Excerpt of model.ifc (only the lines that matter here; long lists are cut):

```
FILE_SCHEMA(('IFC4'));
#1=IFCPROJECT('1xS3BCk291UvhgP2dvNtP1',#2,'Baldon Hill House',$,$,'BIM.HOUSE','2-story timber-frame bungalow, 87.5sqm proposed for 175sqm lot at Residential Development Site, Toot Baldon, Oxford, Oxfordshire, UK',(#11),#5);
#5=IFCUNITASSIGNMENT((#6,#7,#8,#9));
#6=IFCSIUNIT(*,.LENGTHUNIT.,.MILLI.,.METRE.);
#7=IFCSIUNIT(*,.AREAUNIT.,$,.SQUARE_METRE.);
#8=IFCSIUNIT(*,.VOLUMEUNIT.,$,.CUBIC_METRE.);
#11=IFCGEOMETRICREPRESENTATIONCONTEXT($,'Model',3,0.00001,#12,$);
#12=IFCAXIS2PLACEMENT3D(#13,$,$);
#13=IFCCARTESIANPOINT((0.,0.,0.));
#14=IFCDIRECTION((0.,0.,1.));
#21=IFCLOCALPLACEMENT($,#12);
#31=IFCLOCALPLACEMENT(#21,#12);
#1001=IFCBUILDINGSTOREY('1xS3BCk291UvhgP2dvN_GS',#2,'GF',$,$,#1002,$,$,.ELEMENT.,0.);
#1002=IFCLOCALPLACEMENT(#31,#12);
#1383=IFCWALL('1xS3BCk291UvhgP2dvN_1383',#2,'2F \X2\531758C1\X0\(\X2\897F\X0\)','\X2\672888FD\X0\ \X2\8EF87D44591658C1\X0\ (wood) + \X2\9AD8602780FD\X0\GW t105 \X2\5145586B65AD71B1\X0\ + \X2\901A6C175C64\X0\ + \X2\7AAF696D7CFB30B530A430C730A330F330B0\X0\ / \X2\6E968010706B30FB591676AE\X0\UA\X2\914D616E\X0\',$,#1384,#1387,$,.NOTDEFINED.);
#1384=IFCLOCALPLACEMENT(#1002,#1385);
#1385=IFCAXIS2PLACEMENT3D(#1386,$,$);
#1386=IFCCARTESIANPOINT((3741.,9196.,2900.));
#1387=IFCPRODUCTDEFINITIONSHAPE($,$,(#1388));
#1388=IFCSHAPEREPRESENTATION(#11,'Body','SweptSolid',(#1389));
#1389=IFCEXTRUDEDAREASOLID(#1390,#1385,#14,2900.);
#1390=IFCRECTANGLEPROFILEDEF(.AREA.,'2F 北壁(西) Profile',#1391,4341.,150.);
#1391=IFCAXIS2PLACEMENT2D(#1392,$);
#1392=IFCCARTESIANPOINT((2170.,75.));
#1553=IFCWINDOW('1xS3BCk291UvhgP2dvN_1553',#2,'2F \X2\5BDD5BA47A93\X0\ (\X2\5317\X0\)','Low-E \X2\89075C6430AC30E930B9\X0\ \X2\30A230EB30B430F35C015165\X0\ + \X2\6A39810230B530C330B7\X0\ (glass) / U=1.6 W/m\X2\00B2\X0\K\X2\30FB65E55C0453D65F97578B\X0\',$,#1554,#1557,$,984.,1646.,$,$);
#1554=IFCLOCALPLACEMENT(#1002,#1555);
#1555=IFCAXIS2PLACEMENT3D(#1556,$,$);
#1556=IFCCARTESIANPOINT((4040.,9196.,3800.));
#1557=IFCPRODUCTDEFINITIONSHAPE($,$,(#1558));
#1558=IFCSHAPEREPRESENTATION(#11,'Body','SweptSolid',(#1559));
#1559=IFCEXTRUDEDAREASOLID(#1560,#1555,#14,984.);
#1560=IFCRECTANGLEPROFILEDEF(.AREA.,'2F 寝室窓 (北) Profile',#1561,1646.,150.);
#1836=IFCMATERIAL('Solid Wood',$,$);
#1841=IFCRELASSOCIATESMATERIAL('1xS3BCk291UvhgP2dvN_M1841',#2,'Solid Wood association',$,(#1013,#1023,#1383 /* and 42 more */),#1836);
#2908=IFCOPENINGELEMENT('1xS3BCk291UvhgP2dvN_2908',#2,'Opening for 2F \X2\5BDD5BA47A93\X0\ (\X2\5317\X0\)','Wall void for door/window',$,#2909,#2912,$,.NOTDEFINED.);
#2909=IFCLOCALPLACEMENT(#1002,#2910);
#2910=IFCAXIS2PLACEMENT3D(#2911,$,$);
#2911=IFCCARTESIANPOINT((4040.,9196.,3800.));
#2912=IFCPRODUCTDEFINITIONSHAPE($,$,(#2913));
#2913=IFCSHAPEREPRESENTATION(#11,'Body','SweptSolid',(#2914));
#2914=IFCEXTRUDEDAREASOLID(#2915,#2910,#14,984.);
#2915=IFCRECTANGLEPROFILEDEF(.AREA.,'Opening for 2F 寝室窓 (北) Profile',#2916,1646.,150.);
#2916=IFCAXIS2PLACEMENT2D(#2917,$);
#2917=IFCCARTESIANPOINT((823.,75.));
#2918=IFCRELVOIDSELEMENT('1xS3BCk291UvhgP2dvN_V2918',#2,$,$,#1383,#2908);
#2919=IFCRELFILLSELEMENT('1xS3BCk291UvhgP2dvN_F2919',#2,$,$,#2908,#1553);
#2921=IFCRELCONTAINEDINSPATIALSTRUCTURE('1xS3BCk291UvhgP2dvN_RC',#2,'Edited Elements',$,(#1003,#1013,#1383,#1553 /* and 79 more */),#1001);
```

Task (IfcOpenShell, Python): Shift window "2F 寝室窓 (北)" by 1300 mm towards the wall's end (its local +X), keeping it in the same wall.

```python
import ifcopenshell
import ifcopenshell.api.geometry
import ifcopenshell.util.placement

model = ifcopenshell.open("model.ifc")

window = model.by_guid("1xS3BCk291UvhgP2dvN_1553")
opening = window.FillsVoids[0].RelatingOpeningElement
wall = opening.VoidsElements[0].RelatingBuildingElement

wall_matrix = ifcopenshell.util.placement.get_local_placement(wall.ObjectPlacement)
shift = wall_matrix[:3, 0] * 1300.0
before = ifcopenshell.util.placement.get_local_placement(window.ObjectPlacement)[:3, 3].copy()

# The window is not placed relative to its opening, so move both.
for product in (opening, window):
    matrix = ifcopenshell.util.placement.get_local_placement(product.ObjectPlacement)
    matrix[:3, 3] += shift
    ifcopenshell.api.geometry.edit_object_placement(model, product=product, matrix=matrix, is_si=False)

after = ifcopenshell.util.placement.get_local_placement(window.ObjectPlacement)[:3, 3]
print("window moved by", (after - before).round(3) + 0.0)

model.write("model_edited.ifc")
```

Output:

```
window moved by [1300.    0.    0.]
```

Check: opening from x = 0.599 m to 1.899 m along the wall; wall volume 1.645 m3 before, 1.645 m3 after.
